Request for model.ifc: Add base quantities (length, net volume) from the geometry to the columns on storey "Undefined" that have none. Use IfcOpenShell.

First a look at what the model holds.

```python
import ifcopenshell
import ifcopenshell.util.element
import ifcopenshell.util.unit

model = ifcopenshell.open("model.ifc")
print(model.schema)
for unit_type in ("LENGTHUNIT", "AREAUNIT", "VOLUMEUNIT"):
    print(unit_type, ifcopenshell.util.unit.calculate_unit_scale(model, unit_type))
storey = next(s for s in model.by_type("IfcBuildingStorey") if s.Name == "Undefined")
columns = [e for e in ifcopenshell.util.element.get_decomposition(storey) if e.is_a("IfcColumn")]
for e in sorted(columns, key=lambda e: e.id()):
    print(e.id(), e.is_a(), e.Name, list(ifcopenshell.util.element.get_psets(e, qtos_only=True)), sep=" | ")
```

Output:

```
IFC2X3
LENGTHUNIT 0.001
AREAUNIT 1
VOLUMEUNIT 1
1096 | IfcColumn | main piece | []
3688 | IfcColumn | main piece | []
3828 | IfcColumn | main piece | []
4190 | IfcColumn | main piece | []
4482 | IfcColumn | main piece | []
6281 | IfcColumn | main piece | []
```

```python
import ifcopenshell
import ifcopenshell.api.pset
import ifcopenshell.geom
import ifcopenshell.util.element
import ifcopenshell.util.shape
import ifcopenshell.util.unit

model = ifcopenshell.open("model.ifc")
unit_scale = ifcopenshell.util.unit.calculate_unit_scale(model)
volume_scale = ifcopenshell.util.unit.calculate_unit_scale(model, "VOLUMEUNIT")
settings = ifcopenshell.geom.settings()

storey = next(s for s in model.by_type("IfcBuildingStorey") if s.Name == "Undefined")
columns = [e for e in ifcopenshell.util.element.get_decomposition(storey) if e.is_a("IfcColumn")]

for e in sorted(columns, key=lambda e: e.id()):
    if ifcopenshell.util.element.get_psets(e, qtos_only=True, should_inherit=False):
        continue
    # Geometry comes back in metres, in the element's own axes.
    shape = ifcopenshell.geom.create_shape(settings, e)
    values = {
        "Length": ifcopenshell.util.shape.get_z(shape.geometry) / unit_scale,
        "NetVolume": ifcopenshell.util.shape.get_volume(shape.geometry) / volume_scale,
    }
    qto = ifcopenshell.api.pset.add_qto(model, product=e, name="BaseQuantities")
    ifcopenshell.api.pset.edit_qto(model, qto=qto, properties=values)
    print(e.id(), {k: round(v, 3) for k, v in values.items()})

model.write("model_v2.ifc")
```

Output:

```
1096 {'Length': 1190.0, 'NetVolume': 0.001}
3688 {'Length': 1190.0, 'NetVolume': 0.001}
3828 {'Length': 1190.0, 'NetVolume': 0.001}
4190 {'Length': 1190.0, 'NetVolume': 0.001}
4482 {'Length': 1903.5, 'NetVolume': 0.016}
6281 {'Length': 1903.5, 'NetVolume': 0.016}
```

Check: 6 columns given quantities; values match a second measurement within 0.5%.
